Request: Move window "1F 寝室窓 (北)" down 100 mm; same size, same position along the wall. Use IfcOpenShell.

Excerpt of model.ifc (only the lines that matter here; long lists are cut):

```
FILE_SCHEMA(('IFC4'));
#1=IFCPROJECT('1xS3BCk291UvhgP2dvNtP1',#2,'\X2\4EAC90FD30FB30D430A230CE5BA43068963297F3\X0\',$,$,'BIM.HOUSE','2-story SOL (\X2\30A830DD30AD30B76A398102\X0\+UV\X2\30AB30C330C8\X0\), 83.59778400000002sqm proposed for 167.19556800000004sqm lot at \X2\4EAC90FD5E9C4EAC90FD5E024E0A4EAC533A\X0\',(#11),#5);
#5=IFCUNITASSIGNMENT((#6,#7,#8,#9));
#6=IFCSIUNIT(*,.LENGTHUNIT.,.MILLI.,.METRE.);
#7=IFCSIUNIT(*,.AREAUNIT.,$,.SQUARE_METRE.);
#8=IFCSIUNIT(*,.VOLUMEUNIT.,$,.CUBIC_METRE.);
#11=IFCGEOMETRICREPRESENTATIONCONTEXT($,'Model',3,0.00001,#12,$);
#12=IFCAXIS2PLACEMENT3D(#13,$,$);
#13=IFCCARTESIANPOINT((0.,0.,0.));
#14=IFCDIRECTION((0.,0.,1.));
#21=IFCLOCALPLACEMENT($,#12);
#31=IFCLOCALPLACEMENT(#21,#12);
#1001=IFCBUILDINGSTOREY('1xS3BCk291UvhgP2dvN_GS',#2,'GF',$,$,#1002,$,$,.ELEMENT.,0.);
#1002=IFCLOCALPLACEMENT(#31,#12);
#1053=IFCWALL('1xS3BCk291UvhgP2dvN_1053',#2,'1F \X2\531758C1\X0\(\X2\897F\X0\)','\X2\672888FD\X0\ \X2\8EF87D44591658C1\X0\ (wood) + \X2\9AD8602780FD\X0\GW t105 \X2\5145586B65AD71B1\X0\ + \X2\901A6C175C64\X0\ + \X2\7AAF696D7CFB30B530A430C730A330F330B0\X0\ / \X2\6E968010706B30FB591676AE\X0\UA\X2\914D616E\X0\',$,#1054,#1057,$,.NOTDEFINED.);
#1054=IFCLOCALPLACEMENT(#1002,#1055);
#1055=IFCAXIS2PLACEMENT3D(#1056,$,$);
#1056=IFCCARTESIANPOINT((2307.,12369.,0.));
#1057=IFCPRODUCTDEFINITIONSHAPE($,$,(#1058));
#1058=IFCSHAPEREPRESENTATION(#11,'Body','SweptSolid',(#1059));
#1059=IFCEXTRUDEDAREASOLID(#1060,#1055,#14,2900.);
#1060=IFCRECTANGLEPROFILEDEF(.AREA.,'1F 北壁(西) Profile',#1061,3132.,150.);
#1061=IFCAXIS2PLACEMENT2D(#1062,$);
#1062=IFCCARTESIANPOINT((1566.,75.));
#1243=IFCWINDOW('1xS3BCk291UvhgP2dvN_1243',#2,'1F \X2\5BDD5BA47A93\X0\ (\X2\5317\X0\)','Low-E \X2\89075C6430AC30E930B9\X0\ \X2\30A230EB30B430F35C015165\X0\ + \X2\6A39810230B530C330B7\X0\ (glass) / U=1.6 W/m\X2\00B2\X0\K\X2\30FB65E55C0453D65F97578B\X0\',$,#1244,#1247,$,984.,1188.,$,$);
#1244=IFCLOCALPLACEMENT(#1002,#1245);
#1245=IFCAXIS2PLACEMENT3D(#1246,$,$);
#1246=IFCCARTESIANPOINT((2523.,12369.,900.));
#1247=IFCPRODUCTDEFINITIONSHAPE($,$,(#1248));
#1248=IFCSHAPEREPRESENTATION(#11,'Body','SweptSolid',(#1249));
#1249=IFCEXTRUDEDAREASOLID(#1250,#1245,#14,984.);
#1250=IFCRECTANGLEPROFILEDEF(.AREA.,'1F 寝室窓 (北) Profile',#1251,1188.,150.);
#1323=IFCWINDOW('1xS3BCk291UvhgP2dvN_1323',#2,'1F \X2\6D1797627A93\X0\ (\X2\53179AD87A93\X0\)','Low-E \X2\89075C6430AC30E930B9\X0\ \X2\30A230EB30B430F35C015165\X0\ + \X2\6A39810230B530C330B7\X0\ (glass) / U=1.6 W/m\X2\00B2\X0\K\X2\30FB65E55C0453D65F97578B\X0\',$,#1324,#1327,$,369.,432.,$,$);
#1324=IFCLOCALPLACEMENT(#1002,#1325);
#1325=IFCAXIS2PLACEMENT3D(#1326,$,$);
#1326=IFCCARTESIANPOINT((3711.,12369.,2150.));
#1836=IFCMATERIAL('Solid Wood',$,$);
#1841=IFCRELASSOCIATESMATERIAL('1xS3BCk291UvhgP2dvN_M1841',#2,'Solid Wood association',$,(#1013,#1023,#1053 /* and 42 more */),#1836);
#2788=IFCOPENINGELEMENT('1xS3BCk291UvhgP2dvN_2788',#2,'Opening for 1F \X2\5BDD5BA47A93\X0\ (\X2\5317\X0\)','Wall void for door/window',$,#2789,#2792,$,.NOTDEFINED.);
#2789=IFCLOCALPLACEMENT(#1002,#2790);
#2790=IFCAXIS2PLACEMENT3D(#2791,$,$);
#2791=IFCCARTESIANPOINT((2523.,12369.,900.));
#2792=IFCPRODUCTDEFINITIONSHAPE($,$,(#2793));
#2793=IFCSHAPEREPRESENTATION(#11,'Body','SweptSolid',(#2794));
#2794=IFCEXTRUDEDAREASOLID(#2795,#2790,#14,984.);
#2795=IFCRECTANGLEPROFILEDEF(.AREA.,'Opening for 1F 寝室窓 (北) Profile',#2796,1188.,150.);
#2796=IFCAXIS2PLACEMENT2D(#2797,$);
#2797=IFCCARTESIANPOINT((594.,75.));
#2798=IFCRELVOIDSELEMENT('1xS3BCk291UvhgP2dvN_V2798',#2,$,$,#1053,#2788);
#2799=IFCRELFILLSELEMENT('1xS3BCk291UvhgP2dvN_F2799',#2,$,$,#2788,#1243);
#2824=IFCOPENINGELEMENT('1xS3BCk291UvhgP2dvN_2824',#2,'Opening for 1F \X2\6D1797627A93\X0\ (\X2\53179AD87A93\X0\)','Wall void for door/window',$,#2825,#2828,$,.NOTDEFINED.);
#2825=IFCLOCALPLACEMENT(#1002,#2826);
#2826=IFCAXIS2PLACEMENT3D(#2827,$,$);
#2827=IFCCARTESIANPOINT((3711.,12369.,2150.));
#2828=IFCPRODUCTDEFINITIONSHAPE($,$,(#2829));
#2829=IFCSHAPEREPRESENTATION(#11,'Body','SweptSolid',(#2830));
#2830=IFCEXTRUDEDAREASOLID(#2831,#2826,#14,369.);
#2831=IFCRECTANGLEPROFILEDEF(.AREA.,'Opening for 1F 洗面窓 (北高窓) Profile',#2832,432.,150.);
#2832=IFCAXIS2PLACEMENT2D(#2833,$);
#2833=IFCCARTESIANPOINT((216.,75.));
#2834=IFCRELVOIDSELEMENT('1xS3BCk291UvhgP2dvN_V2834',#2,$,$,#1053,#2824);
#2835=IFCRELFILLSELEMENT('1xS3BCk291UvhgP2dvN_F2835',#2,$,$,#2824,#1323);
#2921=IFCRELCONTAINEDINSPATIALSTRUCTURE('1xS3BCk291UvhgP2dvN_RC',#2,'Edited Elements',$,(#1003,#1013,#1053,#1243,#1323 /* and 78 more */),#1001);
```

```python
import numpy as np
import ifcopenshell
import ifcopenshell.api.geometry
import ifcopenshell.util.placement
import ifcopenshell.util.unit

model = ifcopenshell.open("model.ifc")
unit_scale = ifcopenshell.util.unit.calculate_unit_scale(model)

window = model.by_guid("1xS3BCk291UvhgP2dvN_1243")
opening = window.FillsVoids[0].RelatingOpeningElement
dz = -0.1 / unit_scale

shift = np.array([0.0, 0.0, dz])
# The window is not placed relative to its opening, so move both.
for product in (opening, window):
    matrix = ifcopenshell.util.placement.get_local_placement(product.ObjectPlacement)
    matrix[:3, 3] += shift
    ifcopenshell.api.geometry.edit_object_placement(model, product=product, matrix=matrix, is_si=False)

print(f"moved by {dz * unit_scale:+.3f} m")

model.write("model_edited.ifc")
```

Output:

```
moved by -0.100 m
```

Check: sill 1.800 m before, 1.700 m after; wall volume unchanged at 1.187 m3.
